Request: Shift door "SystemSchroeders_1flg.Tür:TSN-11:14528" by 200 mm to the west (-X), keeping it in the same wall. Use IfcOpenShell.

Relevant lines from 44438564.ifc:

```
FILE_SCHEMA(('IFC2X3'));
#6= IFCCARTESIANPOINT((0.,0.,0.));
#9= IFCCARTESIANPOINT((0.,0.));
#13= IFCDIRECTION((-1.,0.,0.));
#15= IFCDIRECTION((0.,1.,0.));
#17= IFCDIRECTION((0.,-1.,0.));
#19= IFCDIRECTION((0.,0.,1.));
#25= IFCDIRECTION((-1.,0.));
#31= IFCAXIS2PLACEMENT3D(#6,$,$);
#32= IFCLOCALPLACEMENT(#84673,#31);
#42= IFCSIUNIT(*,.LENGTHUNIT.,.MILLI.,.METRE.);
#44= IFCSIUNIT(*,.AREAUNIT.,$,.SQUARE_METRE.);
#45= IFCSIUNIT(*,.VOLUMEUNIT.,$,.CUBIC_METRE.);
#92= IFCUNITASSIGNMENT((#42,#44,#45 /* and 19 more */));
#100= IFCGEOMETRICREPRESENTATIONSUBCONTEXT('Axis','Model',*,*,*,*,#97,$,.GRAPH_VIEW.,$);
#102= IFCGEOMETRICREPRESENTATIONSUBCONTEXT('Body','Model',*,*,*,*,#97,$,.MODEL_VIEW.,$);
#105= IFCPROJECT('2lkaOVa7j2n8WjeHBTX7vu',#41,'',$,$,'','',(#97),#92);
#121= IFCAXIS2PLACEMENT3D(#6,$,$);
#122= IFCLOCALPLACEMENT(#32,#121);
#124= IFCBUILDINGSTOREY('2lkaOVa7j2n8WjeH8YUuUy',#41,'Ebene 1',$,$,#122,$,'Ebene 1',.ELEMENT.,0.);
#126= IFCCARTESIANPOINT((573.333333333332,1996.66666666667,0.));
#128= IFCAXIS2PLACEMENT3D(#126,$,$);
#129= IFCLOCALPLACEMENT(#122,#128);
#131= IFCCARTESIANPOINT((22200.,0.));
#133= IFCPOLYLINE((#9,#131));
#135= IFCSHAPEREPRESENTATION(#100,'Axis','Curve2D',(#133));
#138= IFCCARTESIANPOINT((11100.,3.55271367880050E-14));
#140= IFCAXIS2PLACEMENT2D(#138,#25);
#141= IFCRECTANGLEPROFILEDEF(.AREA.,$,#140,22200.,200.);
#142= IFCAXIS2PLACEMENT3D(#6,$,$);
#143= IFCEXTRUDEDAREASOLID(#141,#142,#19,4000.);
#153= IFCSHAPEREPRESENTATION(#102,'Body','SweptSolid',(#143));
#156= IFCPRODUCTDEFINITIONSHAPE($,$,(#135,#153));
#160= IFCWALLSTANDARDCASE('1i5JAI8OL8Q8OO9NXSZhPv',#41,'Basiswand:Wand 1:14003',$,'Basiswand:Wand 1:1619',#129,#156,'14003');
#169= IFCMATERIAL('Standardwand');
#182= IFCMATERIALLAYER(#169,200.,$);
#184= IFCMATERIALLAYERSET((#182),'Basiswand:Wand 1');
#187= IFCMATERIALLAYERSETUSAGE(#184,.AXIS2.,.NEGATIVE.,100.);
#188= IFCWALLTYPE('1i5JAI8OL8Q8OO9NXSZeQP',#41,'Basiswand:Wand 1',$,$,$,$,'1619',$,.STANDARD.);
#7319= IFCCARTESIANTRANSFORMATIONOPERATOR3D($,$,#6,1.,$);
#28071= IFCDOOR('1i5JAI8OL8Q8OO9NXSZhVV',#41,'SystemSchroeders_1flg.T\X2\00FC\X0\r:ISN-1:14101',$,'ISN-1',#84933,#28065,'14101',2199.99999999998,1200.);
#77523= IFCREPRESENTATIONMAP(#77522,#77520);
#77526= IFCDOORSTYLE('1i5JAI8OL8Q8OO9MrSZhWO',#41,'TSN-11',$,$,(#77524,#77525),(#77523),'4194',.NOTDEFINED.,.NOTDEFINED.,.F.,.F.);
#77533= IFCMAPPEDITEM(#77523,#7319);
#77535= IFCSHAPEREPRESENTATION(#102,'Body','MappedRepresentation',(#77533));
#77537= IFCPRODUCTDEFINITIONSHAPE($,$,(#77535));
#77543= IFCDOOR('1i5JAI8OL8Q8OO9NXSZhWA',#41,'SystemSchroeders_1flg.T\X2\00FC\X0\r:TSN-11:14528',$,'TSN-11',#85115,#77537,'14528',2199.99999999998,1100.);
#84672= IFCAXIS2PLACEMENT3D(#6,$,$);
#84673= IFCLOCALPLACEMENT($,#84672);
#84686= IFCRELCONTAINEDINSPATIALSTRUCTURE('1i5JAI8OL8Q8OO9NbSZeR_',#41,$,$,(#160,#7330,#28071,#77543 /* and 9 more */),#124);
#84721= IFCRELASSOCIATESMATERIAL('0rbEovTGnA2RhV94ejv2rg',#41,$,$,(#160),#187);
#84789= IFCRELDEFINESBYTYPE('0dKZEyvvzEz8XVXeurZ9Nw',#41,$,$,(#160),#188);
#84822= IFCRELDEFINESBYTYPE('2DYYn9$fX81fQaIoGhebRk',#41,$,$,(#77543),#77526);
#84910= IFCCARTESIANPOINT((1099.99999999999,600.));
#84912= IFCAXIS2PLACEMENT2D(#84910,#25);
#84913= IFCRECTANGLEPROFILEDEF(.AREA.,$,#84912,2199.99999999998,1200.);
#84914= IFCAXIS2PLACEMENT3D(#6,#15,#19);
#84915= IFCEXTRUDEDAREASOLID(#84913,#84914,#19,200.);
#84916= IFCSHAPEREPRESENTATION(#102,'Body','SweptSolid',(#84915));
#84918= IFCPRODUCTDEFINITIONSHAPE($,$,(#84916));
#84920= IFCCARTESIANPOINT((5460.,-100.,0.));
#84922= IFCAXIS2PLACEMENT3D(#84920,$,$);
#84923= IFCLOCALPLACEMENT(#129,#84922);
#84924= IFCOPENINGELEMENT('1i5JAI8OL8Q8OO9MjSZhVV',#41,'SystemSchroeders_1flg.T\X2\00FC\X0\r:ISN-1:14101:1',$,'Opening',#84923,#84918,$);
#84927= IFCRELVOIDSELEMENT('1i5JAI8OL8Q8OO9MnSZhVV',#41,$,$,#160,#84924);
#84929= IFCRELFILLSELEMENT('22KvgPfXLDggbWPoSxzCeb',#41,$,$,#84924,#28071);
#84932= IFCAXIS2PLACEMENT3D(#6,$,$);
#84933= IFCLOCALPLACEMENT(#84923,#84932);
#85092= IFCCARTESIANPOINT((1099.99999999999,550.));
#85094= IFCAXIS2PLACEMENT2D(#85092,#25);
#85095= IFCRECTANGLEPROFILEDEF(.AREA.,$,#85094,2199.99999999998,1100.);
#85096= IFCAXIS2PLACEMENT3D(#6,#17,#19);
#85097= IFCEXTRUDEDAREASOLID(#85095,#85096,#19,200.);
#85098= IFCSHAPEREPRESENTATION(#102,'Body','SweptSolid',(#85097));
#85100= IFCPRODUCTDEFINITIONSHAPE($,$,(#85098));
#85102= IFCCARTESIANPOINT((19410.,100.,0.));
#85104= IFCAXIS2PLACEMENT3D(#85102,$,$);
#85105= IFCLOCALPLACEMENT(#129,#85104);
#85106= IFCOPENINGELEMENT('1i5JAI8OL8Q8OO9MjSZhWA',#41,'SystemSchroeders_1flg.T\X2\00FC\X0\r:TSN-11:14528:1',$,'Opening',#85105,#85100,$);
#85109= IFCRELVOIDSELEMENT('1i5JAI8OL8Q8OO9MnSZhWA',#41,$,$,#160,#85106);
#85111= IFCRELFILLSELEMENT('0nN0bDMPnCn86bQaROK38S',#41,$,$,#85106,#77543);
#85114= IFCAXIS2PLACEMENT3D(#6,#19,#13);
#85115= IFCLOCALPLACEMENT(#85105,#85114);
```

```python
import ifcopenshell
import ifcopenshell.api.geometry
import ifcopenshell.util.placement

model = ifcopenshell.open("44438564.ifc")

door = model.by_guid("1i5JAI8OL8Q8OO9NXSZhWA")
opening = door.FillsVoids[0].RelatingOpeningElement
wall = opening.VoidsElements[0].RelatingBuildingElement

wall_matrix = ifcopenshell.util.placement.get_local_placement(wall.ObjectPlacement)
shift = wall_matrix[:3, 0] * -200.0
before = ifcopenshell.util.placement.get_local_placement(door.ObjectPlacement)[:3, 3].copy()

# The door is placed relative to its opening, so it follows when the opening moves.
matrix = ifcopenshell.util.placement.get_local_placement(opening.ObjectPlacement)
matrix[:3, 3] += shift
ifcopenshell.api.geometry.edit_object_placement(
    model, product=opening, matrix=matrix, is_si=False, should_transform_children=True
)

after = ifcopenshell.util.placement.get_local_placement(door.ObjectPlacement)[:3, 3]
print("door moved by", (after - before).round(3) + 0.0)

model.write("44438564_updated.ifc")
```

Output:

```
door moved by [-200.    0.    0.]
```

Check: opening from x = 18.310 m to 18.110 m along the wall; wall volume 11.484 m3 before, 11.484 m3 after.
